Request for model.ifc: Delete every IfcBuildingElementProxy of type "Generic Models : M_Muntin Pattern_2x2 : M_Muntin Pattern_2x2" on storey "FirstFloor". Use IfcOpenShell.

First a look at what the model holds.

```python
import ifcopenshell
import ifcopenshell.util.element

model = ifcopenshell.open("model.ifc")
print(model.schema)
storey = next(s for s in model.by_type("IfcBuildingStorey") if s.Name == "FirstFloor")
proxies = [e for e in ifcopenshell.util.element.get_decomposition(storey) if e.is_a("IfcBuildingElementProxy")]
seen = {}
for e in proxies:
    element_type = ifcopenshell.util.element.get_type(e)
    name = element_type.Name if element_type not in (None, e) else None
    seen[name] = seen.get(name, 0) + 1
for name, count in sorted(seen.items(), key=str):
    print(count, "x", name)
```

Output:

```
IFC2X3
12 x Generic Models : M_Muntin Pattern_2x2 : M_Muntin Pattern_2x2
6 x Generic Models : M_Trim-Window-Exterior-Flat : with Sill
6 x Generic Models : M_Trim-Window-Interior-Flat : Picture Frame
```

```python
import ifcopenshell
import ifcopenshell.api.root
import ifcopenshell.util.element

model = ifcopenshell.open("model.ifc")

storey = next(s for s in model.by_type("IfcBuildingStorey") if s.Name == "FirstFloor")
proxies = [e for e in ifcopenshell.util.element.get_decomposition(storey) if e.is_a("IfcBuildingElementProxy")]
targets = [e for e in proxies if (t := ifcopenshell.util.element.get_type(e)) not in (None, e) and t.Name == "Generic Models : M_Muntin Pattern_2x2 : M_Muntin Pattern_2x2"]

for e in targets:
    ifcopenshell.api.root.remove_product(model, product=e)
print(len(targets), "removed")

model.write("model_edited.ifc")
```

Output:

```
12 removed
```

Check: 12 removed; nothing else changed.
